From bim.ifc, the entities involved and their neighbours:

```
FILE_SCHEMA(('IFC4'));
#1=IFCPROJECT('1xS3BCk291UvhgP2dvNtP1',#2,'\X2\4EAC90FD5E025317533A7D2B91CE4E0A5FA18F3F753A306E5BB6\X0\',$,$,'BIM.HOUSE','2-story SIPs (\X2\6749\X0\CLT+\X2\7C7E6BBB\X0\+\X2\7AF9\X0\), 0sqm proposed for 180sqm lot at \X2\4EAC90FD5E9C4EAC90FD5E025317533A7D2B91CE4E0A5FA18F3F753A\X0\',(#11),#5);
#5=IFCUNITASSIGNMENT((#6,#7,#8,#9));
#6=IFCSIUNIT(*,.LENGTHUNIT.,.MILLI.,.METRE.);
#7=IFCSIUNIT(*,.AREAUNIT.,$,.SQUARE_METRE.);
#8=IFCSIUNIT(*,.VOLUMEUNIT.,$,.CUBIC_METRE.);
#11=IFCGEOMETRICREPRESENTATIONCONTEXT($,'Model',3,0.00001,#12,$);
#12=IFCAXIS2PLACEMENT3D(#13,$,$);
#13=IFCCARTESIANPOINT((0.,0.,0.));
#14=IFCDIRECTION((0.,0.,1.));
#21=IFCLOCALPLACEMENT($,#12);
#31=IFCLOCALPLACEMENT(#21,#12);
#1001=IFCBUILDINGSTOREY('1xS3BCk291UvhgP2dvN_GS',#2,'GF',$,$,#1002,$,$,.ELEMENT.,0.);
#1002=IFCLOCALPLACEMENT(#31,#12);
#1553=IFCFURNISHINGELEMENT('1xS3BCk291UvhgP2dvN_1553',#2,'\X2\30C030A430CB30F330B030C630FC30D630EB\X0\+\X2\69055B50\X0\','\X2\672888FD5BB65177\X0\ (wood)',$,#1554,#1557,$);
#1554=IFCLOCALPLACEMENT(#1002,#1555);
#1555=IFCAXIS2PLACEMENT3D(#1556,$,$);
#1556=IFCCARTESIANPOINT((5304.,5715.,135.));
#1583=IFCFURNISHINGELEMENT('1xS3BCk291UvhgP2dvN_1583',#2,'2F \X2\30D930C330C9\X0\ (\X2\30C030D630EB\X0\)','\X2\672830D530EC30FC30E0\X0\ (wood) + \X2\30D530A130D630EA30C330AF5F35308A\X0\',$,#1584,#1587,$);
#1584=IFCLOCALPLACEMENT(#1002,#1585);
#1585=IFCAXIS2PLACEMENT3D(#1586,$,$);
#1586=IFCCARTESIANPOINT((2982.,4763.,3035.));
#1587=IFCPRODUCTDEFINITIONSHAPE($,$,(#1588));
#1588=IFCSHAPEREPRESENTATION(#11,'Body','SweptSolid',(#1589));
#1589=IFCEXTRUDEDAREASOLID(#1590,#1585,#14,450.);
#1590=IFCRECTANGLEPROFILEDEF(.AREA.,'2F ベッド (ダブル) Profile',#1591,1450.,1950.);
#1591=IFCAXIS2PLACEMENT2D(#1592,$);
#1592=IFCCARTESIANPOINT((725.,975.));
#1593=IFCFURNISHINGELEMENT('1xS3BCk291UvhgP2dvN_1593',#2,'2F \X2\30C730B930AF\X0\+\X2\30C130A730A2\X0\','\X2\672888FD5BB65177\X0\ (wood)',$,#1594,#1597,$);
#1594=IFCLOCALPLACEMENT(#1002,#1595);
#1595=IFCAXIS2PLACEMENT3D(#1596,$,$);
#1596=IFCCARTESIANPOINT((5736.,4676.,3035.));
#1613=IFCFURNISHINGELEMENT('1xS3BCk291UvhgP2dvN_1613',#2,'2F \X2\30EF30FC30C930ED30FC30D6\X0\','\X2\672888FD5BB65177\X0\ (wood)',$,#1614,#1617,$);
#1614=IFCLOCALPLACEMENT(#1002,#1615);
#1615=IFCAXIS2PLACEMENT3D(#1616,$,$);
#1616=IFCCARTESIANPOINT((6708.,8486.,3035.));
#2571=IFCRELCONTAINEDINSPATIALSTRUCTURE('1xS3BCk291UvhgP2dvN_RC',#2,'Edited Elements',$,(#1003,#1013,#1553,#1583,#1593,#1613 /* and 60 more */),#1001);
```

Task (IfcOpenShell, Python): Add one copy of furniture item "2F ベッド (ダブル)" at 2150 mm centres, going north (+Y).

```python
import numpy as np
import ifcopenshell
import ifcopenshell.api.geometry
import ifcopenshell.api.root
import ifcopenshell.util.element
import ifcopenshell.util.placement

model = ifcopenshell.open("bim.ifc")


def reuse_history(source, copy):
    """copy_class also copies each property set's owner history, people and application; keep the originals."""
    for rel in copy.IsDefinedBy:
        if rel.is_a("IfcRelDefinesByProperties") and (history := rel.RelatingPropertyDefinition.OwnerHistory):
            rel.RelatingPropertyDefinition.OwnerHistory = source.OwnerHistory
            ifcopenshell.util.element.remove_deep2(model, history)


source = model.by_guid("1xS3BCk291UvhgP2dvN_1583")
base = ifcopenshell.util.placement.get_local_placement(source.ObjectPlacement)
step = np.array([0.0, 1.0, 0.0]) * 2150.0

for i in range(1, 2):
    copy = ifcopenshell.api.root.copy_class(model, product=source)
    copy.Representation = ifcopenshell.util.element.copy_deep(
        model, source.Representation, exclude=["IfcGeometricRepresentationContext", "IfcRepresentationMap"]
    )
    reuse_history(source, copy)
    matrix = base.copy()
    matrix[:3, 3] += i * step
    print("added at", matrix[:3, 3].round(3) + 0.0)
    ifcopenshell.api.geometry.edit_object_placement(model, product=copy, matrix=matrix, is_si=False)

model.write("bim_edited.ifc")
```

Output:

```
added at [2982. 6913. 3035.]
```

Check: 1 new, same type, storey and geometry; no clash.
